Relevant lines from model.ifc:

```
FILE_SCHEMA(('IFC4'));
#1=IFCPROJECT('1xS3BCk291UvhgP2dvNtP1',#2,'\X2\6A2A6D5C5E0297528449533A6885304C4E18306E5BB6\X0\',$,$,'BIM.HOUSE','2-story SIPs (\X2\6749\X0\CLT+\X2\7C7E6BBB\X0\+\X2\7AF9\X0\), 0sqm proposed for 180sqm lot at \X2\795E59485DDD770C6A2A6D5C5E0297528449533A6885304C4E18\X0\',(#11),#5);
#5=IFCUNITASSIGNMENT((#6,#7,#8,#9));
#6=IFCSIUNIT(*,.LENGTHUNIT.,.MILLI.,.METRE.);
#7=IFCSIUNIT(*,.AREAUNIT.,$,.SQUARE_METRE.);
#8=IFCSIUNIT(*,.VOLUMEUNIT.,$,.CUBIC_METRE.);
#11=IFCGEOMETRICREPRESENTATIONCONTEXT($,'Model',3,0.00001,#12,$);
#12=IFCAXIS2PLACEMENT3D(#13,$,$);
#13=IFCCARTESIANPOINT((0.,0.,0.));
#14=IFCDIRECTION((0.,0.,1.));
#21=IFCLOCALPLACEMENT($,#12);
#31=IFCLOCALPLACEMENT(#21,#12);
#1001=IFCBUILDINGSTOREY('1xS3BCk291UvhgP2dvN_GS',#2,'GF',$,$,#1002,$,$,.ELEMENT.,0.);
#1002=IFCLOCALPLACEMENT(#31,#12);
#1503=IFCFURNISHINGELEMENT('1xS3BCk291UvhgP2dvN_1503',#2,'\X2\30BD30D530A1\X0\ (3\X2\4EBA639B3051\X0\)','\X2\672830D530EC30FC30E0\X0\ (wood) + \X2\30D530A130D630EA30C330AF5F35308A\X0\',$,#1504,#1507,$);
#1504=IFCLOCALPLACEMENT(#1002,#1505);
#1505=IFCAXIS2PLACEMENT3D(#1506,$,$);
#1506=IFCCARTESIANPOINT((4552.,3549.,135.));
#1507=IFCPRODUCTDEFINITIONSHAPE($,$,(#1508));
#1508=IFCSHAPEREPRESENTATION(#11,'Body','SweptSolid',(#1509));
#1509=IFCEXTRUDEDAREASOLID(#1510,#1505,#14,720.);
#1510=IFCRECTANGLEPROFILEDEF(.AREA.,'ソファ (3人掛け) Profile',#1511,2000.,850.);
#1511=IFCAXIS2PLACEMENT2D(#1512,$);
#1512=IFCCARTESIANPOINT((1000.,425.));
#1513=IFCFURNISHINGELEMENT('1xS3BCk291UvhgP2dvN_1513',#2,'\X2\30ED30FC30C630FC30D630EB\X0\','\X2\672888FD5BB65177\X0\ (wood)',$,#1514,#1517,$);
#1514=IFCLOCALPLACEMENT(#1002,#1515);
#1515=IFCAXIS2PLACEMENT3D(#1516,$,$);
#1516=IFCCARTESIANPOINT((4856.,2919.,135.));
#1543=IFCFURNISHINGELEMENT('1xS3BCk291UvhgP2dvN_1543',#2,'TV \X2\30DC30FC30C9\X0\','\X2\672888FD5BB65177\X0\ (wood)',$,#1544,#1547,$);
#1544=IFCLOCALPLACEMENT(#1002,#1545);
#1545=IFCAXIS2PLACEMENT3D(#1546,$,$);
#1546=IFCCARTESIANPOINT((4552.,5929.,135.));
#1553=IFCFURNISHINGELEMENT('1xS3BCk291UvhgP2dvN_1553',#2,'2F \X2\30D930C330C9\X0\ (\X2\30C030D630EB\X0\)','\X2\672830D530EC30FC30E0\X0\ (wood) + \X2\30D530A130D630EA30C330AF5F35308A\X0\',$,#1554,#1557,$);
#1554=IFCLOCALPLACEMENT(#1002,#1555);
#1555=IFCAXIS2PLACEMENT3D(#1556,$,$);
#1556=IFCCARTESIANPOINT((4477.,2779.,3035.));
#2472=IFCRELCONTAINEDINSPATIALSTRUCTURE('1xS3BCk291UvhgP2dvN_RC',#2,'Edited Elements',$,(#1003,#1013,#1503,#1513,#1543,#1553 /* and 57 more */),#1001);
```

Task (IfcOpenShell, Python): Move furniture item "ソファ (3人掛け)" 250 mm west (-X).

```python
import ifcopenshell
import ifcopenshell.api.geometry
import ifcopenshell.util.placement

model = ifcopenshell.open("model.ifc")

item = model.by_guid("1xS3BCk291UvhgP2dvN_1503")
matrix = ifcopenshell.util.placement.get_local_placement(item.ObjectPlacement)
matrix[0, 3] -= 250.0
ifcopenshell.api.geometry.edit_object_placement(model, product=item, matrix=matrix, is_si=False)

print(ifcopenshell.util.placement.get_local_placement(item.ObjectPlacement).round(3) + 0.0)

model.write("model_updated.ifc")
```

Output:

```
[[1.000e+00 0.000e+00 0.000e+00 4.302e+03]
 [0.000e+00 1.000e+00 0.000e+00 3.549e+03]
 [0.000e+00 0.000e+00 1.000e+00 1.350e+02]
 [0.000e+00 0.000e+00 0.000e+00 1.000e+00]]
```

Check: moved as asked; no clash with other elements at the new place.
